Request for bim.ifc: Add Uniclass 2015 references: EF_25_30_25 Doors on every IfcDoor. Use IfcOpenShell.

First a look at what the model holds.

```python
import ifcopenshell

model = ifcopenshell.open("bim.ifc")
print(model.schema)
print("classifications:", [c.Name for c in model.by_type("IfcClassification")])
for ifc_class in ("IfcDoor", "IfcRoof", "IfcStair", "IfcWall", "IfcWindow"):
    print(ifc_class, len(model.by_type(ifc_class)))
```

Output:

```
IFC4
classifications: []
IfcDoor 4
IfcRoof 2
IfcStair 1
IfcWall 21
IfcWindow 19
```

```python
import ifcopenshell
import ifcopenshell.api.classification

model = ifcopenshell.open("bim.ifc")

system = ifcopenshell.api.classification.add_classification(model, classification="Uniclass 2015")

codes = {
    "IfcDoor": ("EF_25_30_25", "Doors"),
}
for ifc_class, (code, name) in codes.items():
    products = model.by_type(ifc_class)
    ifcopenshell.api.classification.add_reference(
        model, products=products, classification=system, identification=code, name=name
    )
    print(code, len(products))

model.write("bim_edited.ifc")
```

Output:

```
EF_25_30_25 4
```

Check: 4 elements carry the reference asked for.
